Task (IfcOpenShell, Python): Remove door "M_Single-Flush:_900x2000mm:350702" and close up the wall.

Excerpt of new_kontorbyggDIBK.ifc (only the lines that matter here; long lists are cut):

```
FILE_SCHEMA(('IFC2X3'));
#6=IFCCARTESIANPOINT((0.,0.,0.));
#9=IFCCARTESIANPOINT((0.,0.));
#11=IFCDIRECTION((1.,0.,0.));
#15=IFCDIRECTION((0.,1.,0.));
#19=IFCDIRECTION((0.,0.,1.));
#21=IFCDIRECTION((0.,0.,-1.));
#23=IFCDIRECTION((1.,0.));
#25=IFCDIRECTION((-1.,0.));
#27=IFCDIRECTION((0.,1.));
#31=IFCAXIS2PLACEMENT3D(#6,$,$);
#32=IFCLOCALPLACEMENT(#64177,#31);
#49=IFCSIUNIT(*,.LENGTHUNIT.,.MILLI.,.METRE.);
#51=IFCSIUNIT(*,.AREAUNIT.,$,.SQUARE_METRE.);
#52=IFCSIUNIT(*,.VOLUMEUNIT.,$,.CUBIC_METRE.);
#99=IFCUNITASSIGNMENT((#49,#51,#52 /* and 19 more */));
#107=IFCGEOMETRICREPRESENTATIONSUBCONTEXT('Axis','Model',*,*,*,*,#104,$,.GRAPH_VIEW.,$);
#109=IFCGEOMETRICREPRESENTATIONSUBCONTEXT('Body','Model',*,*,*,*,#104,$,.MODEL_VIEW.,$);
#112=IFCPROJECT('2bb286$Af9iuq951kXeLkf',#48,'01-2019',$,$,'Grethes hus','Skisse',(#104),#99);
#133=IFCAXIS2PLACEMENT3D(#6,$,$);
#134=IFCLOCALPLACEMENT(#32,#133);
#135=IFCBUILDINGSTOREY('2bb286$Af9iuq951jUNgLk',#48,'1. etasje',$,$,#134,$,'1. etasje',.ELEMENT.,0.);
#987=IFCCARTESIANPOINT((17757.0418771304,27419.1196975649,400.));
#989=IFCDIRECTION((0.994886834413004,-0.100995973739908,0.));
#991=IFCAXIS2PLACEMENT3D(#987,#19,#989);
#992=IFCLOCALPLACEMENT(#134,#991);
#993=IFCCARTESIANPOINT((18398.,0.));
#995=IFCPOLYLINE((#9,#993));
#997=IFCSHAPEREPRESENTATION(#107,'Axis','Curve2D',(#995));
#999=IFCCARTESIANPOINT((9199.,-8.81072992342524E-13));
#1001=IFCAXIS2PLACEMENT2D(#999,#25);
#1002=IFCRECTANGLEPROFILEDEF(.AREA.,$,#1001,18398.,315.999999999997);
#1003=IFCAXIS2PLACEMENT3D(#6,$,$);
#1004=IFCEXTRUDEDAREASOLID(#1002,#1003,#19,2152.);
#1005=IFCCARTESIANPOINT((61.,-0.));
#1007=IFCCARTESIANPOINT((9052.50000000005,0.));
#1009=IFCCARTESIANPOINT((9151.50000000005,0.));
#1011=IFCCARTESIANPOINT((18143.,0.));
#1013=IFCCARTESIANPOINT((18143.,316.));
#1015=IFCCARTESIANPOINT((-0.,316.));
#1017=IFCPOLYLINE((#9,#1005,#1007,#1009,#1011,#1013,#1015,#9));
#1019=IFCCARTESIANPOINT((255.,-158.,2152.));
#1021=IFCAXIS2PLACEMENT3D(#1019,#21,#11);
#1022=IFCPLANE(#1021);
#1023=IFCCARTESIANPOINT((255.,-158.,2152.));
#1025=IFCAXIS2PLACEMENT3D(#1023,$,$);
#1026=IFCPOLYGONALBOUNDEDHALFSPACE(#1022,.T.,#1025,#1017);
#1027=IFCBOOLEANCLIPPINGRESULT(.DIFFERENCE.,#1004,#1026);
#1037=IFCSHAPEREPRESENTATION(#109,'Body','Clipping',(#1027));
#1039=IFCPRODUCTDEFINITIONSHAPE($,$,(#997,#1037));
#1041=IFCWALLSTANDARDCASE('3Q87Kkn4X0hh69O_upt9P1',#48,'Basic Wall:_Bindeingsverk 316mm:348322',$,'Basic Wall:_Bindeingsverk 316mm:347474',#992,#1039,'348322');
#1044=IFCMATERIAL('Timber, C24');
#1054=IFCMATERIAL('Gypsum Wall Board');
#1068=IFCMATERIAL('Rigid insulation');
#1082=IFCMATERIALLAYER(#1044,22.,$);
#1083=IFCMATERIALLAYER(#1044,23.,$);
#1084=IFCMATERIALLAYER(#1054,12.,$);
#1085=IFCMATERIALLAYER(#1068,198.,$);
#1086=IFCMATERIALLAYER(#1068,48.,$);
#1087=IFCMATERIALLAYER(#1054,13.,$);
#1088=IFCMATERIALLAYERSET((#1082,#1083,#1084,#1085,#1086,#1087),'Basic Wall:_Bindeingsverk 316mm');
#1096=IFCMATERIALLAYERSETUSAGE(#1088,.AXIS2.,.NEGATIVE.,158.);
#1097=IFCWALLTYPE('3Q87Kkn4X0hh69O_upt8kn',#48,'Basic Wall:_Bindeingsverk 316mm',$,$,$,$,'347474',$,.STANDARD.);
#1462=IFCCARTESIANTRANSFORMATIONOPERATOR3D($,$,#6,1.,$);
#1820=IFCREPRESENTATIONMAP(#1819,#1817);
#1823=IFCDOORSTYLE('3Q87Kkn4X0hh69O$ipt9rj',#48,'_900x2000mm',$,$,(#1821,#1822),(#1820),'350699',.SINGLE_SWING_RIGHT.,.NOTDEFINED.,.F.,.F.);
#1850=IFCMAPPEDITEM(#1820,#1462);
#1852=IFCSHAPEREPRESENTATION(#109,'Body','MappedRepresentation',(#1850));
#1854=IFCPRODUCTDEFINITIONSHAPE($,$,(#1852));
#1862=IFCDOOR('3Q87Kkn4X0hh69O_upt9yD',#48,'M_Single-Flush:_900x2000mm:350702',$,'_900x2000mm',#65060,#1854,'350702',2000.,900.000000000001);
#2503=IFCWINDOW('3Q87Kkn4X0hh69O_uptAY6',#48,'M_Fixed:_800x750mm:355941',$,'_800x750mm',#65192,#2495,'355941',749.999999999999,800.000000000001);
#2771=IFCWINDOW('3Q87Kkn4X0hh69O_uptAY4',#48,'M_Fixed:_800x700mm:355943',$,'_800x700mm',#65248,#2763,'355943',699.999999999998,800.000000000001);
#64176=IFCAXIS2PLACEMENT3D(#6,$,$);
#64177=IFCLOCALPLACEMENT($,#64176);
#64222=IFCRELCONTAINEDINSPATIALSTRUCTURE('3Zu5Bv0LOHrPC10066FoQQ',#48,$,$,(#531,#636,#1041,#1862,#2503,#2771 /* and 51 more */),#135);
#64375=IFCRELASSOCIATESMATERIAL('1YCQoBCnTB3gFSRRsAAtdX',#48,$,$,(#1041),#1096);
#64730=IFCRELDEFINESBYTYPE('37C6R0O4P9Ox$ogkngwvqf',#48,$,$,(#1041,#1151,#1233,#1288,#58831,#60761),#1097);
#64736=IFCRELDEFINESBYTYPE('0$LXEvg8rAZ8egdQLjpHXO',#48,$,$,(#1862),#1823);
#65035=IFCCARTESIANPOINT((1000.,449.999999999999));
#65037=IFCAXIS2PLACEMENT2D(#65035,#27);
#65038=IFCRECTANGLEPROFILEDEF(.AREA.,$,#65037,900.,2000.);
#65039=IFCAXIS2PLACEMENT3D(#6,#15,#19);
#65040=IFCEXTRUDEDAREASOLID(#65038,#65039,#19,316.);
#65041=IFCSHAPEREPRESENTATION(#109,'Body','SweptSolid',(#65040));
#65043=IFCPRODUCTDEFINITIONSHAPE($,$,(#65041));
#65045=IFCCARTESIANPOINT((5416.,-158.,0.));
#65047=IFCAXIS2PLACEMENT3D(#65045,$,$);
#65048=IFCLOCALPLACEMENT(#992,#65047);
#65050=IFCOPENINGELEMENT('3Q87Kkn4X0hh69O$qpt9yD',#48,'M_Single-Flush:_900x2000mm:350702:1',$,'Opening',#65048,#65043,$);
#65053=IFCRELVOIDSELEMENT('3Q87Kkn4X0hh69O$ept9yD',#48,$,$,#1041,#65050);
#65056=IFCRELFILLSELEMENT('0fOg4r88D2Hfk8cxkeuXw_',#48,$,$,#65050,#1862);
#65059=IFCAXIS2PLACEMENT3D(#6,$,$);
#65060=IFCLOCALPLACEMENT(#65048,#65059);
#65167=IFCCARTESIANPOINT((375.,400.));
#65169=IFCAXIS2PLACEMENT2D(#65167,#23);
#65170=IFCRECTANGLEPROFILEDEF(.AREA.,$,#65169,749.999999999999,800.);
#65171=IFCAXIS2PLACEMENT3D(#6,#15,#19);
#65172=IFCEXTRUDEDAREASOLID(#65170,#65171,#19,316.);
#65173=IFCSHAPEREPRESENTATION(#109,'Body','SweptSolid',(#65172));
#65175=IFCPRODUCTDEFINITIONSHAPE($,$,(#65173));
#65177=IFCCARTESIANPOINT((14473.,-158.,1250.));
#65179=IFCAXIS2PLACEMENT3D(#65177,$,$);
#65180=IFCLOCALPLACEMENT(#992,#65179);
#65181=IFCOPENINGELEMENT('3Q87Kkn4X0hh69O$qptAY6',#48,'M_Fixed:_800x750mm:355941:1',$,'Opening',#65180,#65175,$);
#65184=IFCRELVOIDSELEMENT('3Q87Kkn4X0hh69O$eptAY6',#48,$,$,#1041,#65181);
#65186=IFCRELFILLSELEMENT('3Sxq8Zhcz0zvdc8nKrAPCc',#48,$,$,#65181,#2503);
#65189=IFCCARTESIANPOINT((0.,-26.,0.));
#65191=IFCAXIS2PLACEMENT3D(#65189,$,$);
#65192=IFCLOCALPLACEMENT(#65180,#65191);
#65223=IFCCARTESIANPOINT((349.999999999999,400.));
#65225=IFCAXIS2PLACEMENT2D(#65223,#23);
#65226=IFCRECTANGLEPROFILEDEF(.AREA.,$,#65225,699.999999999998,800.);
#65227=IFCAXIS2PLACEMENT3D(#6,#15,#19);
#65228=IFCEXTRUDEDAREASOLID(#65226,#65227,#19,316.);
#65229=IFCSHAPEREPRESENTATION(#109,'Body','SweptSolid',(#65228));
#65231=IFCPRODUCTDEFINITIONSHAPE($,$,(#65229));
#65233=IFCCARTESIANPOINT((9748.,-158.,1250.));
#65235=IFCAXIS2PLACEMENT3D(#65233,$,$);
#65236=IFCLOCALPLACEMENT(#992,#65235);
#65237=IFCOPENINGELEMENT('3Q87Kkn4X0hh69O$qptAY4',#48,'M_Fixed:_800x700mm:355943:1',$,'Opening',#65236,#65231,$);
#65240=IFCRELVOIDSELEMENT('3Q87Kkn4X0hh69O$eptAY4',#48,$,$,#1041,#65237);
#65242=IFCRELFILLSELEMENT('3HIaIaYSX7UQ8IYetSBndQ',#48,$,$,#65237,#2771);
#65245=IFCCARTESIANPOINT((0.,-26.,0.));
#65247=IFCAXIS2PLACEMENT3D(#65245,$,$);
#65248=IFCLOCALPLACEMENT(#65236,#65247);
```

```python
import ifcopenshell
import ifcopenshell.api.feature
import ifcopenshell.api.root
import ifcopenshell.geom
import ifcopenshell.util.shape

model = ifcopenshell.open("new_kontorbyggDIBK.ifc")
settings = ifcopenshell.geom.settings()


def volume(element):
    """Net volume in cubic metres, openings subtracted."""
    shape = ifcopenshell.geom.create_shape(settings, element)
    return ifcopenshell.util.shape.get_volume(shape.geometry)


door = model.by_guid("3Q87Kkn4X0hh69O_upt9yD")
opening = door.FillsVoids[0].RelatingOpeningElement
wall = opening.VoidsElements[0].RelatingBuildingElement
before = volume(wall)

ifcopenshell.api.root.remove_product(model, product=door)
ifcopenshell.api.feature.remove_feature(model, feature=opening)

after = volume(wall)

print(f"wall volume {before:.3f} -> {after:.3f} m3")

model.write("new_kontorbyggDIBK_rev.ifc")
```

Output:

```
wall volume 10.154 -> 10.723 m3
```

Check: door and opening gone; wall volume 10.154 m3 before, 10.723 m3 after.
